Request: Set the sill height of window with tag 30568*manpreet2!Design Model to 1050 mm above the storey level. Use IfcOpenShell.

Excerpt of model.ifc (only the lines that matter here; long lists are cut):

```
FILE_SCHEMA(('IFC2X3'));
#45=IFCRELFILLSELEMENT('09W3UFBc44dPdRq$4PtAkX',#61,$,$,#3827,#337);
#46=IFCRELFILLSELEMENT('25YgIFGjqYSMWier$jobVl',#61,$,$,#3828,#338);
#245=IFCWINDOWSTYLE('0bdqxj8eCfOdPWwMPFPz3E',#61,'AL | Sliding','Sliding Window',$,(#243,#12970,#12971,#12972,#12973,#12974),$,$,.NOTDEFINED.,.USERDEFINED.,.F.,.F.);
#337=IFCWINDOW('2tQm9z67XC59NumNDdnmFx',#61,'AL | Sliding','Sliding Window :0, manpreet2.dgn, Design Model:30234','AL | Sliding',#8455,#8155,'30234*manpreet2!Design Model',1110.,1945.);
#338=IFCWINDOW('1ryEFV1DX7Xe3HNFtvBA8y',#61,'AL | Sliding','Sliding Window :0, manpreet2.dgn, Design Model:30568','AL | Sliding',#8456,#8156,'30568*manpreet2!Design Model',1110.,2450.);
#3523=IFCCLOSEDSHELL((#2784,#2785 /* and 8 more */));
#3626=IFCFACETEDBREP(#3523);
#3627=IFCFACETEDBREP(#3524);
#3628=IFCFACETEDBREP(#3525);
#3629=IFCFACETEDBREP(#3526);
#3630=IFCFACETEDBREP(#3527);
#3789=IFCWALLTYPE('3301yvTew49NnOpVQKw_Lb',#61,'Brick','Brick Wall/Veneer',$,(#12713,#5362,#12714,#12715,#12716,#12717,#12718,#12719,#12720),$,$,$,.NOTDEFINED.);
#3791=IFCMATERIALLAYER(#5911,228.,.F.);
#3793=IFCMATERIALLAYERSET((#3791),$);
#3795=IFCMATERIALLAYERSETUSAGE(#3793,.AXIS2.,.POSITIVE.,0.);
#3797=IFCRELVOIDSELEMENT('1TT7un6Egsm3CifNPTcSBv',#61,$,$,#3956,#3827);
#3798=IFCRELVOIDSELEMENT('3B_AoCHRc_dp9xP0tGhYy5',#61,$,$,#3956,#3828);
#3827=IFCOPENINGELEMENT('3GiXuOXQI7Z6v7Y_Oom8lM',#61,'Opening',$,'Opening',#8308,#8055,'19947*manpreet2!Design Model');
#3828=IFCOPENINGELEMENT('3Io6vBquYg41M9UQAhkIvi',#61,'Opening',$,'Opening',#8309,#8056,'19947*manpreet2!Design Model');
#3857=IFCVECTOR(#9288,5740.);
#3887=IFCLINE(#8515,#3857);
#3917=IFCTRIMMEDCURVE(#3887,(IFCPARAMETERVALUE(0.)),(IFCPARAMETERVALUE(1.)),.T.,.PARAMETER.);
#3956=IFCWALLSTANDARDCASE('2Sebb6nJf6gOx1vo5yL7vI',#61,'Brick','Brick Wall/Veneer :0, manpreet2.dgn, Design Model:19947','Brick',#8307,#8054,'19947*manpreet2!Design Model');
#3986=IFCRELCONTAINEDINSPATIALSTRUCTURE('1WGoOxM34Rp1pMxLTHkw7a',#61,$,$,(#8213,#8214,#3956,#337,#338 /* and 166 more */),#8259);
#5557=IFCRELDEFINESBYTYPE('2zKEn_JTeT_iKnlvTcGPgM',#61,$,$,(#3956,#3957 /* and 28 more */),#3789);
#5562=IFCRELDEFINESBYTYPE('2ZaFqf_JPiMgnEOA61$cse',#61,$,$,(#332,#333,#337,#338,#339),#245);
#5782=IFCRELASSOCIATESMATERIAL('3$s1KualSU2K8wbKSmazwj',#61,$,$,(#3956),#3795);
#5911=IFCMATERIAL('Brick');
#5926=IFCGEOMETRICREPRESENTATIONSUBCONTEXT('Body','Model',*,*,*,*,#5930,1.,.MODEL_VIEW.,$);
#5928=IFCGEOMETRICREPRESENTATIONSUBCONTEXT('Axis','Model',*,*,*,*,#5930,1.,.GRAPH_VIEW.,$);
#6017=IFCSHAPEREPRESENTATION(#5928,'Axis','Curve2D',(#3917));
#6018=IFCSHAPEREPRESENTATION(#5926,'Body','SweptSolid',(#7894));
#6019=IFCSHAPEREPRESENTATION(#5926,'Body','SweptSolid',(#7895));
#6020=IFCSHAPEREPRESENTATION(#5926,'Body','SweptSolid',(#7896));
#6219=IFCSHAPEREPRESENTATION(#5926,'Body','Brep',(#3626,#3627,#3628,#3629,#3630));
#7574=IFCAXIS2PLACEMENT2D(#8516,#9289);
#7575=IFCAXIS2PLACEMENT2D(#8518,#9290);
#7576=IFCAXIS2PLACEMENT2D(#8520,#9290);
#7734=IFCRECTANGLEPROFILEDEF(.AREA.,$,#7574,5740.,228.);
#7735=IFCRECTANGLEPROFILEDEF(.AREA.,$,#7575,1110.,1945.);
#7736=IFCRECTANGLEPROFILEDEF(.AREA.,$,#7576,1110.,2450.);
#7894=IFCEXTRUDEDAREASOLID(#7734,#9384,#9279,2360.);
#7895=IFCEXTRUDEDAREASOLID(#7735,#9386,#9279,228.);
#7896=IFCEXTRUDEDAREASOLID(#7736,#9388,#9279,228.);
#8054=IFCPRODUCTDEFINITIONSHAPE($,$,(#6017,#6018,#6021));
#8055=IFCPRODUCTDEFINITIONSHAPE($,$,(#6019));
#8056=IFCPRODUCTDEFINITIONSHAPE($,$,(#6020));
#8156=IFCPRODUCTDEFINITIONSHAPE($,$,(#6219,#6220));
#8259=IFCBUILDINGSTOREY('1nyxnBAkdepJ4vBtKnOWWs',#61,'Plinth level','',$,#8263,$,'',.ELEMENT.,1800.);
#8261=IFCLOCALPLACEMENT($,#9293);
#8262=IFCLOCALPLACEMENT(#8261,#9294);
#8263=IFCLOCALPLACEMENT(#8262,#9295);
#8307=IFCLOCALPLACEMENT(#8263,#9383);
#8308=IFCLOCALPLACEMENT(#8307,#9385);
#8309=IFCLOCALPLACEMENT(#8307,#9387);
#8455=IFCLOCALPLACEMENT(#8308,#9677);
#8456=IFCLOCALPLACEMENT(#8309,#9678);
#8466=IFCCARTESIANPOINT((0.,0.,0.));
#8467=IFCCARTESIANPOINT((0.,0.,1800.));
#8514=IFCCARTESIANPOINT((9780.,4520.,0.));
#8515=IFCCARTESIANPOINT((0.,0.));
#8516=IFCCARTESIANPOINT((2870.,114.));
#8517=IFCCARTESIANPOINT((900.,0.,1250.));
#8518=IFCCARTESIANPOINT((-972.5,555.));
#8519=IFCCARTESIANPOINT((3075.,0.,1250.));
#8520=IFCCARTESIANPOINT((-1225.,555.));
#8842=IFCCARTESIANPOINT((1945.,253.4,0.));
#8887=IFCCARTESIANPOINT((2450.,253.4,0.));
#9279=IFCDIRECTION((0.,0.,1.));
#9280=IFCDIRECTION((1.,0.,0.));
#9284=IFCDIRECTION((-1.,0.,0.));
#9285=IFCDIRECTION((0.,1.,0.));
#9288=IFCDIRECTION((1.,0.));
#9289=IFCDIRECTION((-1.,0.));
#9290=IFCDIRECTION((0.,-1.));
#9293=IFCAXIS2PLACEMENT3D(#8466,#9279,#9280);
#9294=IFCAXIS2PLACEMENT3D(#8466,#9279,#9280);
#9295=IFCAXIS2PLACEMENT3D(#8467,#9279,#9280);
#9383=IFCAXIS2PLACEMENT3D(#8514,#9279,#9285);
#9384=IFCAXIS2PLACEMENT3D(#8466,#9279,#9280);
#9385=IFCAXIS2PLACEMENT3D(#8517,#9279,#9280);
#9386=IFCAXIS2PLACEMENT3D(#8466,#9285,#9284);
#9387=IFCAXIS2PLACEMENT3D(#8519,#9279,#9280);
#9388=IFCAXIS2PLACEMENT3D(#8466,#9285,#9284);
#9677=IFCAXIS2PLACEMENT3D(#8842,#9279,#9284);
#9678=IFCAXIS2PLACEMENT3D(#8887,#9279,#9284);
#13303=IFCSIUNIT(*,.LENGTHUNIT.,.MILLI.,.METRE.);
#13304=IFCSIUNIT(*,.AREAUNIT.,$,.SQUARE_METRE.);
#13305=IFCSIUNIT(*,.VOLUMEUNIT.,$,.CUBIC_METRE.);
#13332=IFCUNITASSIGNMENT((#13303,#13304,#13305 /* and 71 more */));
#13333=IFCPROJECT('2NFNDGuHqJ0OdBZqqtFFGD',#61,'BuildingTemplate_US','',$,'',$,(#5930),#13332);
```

```python
import numpy as np
import ifcopenshell
import ifcopenshell.api.geometry
import ifcopenshell.geom
import ifcopenshell.util.element
import ifcopenshell.util.placement
import ifcopenshell.util.shape
import ifcopenshell.util.unit

model = ifcopenshell.open("model.ifc")
unit_scale = ifcopenshell.util.unit.calculate_unit_scale(model)

window = model.by_id(338)
opening = window.FillsVoids[0].RelatingOpeningElement
storey = ifcopenshell.util.element.get_container(window, ifc_class="IfcBuildingStorey")
level = ifcopenshell.util.placement.get_local_placement(storey.ObjectPlacement)[2, 3]

# The opening's origin need not be at the sill, so measure its lowest point.
shape = ifcopenshell.geom.create_shape(ifcopenshell.geom.settings(), opening)
bottom = ifcopenshell.util.shape.get_shape_bottom_elevation(shape, shape.geometry) / unit_scale
dz = level + 1050.0 - bottom

shift = np.array([0.0, 0.0, dz])
# The window is placed relative to its opening, so it follows when the opening moves.
matrix = ifcopenshell.util.placement.get_local_placement(opening.ObjectPlacement)
matrix[:3, 3] += shift
ifcopenshell.api.geometry.edit_object_placement(
    model, product=opening, matrix=matrix, is_si=False, should_transform_children=True
)

print(f"moved by {dz * unit_scale:+.3f} m")

model.write("model_v2.ifc")
```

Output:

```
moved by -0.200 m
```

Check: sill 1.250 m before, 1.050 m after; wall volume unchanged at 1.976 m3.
